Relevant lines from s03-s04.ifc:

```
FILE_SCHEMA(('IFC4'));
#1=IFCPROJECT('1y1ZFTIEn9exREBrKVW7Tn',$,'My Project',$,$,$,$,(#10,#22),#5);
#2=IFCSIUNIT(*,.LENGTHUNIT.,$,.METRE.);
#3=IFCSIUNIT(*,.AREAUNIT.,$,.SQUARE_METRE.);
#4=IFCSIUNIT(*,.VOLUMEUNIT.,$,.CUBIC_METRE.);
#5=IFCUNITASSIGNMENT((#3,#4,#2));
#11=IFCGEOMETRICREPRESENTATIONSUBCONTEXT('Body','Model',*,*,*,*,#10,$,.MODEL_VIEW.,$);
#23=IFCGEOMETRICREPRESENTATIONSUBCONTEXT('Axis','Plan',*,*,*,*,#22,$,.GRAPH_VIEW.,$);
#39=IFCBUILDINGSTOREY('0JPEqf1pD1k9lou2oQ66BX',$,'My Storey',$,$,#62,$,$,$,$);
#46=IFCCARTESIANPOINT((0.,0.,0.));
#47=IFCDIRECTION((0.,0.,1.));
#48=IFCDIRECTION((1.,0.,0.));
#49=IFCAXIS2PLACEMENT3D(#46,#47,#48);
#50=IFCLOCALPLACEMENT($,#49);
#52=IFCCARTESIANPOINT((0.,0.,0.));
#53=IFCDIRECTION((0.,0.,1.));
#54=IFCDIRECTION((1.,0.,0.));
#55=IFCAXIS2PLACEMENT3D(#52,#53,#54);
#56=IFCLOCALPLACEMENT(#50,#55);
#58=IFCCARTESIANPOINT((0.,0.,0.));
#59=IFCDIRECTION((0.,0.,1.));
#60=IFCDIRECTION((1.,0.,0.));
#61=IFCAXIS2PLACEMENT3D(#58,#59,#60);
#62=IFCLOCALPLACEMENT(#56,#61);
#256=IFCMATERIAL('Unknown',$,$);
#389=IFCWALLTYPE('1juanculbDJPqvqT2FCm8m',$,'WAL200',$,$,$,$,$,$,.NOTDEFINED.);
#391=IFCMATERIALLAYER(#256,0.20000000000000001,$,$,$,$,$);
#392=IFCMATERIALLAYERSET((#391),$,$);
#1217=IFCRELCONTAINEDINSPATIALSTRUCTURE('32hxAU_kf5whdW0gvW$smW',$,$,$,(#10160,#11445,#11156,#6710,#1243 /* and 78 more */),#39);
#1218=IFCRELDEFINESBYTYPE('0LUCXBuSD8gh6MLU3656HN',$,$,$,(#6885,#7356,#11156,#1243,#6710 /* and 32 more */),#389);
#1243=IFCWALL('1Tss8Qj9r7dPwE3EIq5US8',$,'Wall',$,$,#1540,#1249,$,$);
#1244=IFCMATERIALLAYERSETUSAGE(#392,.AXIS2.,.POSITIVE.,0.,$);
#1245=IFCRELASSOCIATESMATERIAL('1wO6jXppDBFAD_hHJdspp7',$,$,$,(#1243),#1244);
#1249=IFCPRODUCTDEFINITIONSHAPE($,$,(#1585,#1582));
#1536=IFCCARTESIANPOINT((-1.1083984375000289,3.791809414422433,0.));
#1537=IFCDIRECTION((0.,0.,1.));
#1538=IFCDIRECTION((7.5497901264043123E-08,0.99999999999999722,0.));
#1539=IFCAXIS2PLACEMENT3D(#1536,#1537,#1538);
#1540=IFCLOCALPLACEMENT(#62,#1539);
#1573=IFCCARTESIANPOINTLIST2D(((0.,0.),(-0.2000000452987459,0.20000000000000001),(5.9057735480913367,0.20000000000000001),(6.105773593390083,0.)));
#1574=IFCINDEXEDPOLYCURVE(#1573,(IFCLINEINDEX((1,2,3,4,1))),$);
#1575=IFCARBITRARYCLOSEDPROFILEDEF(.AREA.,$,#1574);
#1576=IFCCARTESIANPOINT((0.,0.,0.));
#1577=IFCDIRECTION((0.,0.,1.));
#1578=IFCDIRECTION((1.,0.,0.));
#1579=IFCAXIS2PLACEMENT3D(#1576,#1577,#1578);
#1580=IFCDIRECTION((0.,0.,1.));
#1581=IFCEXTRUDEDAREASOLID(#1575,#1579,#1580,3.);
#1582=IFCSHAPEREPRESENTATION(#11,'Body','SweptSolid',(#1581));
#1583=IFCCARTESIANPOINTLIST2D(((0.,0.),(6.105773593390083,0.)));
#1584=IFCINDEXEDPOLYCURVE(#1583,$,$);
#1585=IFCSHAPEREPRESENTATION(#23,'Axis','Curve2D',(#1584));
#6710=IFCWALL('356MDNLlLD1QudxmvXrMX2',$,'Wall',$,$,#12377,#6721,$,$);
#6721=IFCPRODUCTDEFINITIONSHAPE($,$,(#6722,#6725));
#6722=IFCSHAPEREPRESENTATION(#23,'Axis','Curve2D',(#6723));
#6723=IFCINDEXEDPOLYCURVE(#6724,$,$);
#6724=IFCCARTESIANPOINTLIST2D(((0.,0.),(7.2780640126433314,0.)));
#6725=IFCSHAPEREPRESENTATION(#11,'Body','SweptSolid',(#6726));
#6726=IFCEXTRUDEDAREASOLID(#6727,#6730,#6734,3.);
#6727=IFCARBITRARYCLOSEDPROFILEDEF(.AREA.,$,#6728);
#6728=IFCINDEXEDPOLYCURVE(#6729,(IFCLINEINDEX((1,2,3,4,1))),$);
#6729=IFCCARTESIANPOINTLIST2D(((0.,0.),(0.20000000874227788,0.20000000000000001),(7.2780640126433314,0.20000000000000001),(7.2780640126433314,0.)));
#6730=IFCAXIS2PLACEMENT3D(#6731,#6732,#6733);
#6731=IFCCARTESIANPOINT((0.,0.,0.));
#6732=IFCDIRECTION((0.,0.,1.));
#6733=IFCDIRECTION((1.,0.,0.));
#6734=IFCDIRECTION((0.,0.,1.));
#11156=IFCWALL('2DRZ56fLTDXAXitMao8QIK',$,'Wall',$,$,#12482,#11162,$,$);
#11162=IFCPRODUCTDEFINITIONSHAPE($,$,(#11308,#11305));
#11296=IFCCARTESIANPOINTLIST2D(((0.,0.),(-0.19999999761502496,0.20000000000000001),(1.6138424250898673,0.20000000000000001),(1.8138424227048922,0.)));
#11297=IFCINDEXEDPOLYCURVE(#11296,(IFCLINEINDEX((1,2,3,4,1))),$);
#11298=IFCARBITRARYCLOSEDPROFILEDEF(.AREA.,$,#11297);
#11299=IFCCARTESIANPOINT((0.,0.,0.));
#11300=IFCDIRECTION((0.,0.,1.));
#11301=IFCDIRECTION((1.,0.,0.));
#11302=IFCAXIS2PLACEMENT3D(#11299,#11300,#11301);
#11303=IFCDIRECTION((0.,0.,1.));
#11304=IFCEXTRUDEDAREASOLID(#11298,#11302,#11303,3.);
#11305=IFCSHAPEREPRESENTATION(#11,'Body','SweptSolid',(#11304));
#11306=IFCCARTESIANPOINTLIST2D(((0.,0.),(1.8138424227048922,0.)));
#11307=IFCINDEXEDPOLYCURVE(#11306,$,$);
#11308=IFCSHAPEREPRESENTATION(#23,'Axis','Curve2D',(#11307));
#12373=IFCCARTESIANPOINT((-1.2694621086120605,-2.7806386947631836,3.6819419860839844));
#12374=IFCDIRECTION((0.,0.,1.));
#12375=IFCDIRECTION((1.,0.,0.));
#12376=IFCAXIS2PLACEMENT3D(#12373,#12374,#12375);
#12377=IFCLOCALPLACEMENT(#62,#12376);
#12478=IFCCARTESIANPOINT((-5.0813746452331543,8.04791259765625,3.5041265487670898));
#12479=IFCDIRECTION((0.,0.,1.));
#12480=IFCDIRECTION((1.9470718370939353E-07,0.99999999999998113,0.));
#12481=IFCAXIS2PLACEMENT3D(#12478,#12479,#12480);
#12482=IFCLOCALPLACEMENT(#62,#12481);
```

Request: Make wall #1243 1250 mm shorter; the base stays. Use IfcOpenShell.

```python
import ifcopenshell
import ifcopenshell.geom
import ifcopenshell.util.representation
import ifcopenshell.util.shape

model = ifcopenshell.open("s03-s04.ifc")
settings = ifcopenshell.geom.settings()


def volume(element):
    """Net volume in cubic metres, openings subtracted."""
    shape = ifcopenshell.geom.create_shape(settings, element)
    return ifcopenshell.util.shape.get_volume(shape.geometry)


wall = model.by_guid("1Tss8Qj9r7dPwE3EIq5US8")
before = volume(wall)

body = ifcopenshell.util.representation.get_representation(wall, "Model", "Body")
solid = body.Items[0]
old_height = solid.Depth
solid.Depth -= 1.25
after = volume(wall)

print(f"height {old_height:g} -> {solid.Depth:g}, volume {before:.3f} -> {after:.3f} m3")

model.write("s03-s04_rev.ifc")
```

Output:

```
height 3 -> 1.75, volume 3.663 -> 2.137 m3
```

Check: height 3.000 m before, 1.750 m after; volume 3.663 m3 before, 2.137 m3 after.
